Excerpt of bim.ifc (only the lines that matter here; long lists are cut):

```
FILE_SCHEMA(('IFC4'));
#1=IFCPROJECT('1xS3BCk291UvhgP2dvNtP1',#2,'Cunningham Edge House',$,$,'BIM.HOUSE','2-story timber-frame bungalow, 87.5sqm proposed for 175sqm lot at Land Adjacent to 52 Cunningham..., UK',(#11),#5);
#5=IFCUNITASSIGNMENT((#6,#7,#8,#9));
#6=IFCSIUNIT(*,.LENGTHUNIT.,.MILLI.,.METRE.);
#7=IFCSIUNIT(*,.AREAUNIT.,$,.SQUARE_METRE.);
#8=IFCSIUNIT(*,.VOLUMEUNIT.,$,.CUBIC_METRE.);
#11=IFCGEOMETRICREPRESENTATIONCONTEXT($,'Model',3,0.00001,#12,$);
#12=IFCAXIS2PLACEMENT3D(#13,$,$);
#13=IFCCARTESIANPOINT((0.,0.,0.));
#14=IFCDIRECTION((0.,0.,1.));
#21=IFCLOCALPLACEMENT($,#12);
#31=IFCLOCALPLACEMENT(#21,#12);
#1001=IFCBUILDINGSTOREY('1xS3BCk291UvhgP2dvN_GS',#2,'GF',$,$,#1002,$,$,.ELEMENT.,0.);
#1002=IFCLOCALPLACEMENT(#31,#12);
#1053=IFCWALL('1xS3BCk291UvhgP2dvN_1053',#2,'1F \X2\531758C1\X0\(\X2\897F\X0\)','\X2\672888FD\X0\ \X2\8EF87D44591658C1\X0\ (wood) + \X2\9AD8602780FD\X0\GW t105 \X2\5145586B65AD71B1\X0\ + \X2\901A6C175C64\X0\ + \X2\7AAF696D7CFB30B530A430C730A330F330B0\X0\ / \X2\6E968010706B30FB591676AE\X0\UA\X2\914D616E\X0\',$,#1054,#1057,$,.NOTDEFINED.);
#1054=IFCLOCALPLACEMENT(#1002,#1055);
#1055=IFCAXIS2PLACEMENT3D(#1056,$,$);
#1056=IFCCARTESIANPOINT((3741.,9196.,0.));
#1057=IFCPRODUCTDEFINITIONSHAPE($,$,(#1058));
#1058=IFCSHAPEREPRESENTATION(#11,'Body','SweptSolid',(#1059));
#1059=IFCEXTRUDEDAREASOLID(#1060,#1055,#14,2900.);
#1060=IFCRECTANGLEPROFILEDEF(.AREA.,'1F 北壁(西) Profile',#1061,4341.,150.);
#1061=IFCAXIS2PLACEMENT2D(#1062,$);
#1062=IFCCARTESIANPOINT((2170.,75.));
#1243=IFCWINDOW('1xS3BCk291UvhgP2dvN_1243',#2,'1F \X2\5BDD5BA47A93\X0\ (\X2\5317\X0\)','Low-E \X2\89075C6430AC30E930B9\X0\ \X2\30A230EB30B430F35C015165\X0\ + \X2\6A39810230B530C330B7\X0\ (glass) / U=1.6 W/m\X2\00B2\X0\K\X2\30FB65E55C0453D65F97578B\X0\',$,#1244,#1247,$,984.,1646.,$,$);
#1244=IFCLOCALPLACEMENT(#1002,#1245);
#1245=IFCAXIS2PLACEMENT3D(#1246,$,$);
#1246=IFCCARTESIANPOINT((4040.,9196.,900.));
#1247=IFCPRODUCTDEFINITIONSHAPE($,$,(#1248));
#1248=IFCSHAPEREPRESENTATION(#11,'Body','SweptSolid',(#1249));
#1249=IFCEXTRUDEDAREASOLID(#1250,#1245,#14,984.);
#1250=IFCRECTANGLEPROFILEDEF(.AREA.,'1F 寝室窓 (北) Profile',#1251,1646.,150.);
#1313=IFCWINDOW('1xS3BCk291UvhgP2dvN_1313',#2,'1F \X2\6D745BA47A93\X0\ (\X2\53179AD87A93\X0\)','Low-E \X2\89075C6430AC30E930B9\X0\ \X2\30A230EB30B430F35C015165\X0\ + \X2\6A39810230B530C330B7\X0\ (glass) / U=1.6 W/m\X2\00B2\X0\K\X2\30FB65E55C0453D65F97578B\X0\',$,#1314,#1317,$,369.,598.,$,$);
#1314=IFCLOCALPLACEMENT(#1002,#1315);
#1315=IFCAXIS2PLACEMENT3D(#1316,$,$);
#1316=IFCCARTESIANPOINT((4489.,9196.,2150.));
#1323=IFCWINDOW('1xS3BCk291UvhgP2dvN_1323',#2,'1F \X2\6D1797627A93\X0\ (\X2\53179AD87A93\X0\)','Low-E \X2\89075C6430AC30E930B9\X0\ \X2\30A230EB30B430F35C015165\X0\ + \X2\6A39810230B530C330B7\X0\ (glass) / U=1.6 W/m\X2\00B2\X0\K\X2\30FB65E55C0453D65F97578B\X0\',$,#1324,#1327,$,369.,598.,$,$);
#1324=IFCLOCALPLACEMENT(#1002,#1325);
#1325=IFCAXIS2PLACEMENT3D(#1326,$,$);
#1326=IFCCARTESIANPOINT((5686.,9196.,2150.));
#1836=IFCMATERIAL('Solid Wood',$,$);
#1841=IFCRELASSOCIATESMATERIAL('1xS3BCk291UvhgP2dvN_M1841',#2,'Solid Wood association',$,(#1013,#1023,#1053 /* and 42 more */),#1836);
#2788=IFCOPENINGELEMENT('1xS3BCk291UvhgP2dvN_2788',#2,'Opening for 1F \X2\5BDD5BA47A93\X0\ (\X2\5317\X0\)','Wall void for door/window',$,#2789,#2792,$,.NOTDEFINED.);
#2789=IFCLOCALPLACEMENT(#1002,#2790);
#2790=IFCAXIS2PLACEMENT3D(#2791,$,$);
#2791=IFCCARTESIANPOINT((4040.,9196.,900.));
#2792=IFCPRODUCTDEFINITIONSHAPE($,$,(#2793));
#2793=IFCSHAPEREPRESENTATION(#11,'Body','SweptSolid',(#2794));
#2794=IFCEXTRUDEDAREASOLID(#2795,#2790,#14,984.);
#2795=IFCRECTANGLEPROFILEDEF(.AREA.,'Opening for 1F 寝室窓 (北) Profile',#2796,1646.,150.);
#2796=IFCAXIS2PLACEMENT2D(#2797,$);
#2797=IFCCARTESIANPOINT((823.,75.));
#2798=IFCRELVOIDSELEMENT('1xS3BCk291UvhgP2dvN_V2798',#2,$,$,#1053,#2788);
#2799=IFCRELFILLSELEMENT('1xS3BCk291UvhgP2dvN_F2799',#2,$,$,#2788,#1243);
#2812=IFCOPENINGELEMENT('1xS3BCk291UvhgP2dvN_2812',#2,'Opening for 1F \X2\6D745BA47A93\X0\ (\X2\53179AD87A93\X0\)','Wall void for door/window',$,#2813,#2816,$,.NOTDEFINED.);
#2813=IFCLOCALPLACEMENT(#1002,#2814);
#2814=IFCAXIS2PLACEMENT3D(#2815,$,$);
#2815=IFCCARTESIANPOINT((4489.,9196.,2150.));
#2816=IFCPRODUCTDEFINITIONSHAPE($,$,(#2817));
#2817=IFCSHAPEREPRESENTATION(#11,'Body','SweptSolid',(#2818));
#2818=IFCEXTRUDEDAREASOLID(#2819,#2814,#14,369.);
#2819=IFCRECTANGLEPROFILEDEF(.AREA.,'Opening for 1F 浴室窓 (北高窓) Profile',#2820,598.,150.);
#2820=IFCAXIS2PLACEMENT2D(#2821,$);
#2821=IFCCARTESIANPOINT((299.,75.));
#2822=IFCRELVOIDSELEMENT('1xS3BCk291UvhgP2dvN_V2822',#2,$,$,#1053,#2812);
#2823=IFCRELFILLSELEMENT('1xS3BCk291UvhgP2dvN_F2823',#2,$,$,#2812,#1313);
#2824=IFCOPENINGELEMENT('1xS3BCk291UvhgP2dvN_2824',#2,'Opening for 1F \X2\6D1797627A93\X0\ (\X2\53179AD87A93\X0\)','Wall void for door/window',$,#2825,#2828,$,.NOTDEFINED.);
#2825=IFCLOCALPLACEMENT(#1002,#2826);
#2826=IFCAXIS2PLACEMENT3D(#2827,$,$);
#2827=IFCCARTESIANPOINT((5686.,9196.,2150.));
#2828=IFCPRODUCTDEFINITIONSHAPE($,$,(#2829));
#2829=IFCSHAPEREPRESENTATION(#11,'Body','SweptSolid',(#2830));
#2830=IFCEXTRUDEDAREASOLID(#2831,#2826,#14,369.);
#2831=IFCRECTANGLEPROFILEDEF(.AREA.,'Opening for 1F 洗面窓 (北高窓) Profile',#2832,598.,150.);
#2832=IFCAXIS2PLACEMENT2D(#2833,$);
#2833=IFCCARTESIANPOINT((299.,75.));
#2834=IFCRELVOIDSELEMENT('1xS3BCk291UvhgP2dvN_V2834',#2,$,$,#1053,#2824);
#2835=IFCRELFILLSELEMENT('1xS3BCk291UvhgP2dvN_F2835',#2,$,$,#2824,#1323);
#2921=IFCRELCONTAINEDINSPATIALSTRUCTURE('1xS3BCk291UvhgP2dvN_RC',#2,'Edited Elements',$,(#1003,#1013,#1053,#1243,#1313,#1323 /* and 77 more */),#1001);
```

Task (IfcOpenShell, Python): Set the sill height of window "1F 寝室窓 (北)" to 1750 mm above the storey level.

```python
import numpy as np
import ifcopenshell
import ifcopenshell.api.geometry
import ifcopenshell.geom
import ifcopenshell.util.element
import ifcopenshell.util.placement
import ifcopenshell.util.shape
import ifcopenshell.util.unit

model = ifcopenshell.open("bim.ifc")
unit_scale = ifcopenshell.util.unit.calculate_unit_scale(model)

window = model.by_guid("1xS3BCk291UvhgP2dvN_1243")
opening = window.FillsVoids[0].RelatingOpeningElement
storey = ifcopenshell.util.element.get_container(window, ifc_class="IfcBuildingStorey")
level = ifcopenshell.util.placement.get_local_placement(storey.ObjectPlacement)[2, 3]

# The opening's origin need not be at the sill, so measure its lowest point.
shape = ifcopenshell.geom.create_shape(ifcopenshell.geom.settings(), opening)
bottom = ifcopenshell.util.shape.get_shape_bottom_elevation(shape, shape.geometry) / unit_scale
dz = level + 1750.0 - bottom

shift = np.array([0.0, 0.0, dz])
# The window is not placed relative to its opening, so move both.
for product in (opening, window):
    matrix = ifcopenshell.util.placement.get_local_placement(product.ObjectPlacement)
    matrix[:3, 3] += shift
    ifcopenshell.api.geometry.edit_object_placement(model, product=product, matrix=matrix, is_si=False)

print(f"moved by {dz * unit_scale:+.3f} m")

model.write("bim_v2.ifc")
```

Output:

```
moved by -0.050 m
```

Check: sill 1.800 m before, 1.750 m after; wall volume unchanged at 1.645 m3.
